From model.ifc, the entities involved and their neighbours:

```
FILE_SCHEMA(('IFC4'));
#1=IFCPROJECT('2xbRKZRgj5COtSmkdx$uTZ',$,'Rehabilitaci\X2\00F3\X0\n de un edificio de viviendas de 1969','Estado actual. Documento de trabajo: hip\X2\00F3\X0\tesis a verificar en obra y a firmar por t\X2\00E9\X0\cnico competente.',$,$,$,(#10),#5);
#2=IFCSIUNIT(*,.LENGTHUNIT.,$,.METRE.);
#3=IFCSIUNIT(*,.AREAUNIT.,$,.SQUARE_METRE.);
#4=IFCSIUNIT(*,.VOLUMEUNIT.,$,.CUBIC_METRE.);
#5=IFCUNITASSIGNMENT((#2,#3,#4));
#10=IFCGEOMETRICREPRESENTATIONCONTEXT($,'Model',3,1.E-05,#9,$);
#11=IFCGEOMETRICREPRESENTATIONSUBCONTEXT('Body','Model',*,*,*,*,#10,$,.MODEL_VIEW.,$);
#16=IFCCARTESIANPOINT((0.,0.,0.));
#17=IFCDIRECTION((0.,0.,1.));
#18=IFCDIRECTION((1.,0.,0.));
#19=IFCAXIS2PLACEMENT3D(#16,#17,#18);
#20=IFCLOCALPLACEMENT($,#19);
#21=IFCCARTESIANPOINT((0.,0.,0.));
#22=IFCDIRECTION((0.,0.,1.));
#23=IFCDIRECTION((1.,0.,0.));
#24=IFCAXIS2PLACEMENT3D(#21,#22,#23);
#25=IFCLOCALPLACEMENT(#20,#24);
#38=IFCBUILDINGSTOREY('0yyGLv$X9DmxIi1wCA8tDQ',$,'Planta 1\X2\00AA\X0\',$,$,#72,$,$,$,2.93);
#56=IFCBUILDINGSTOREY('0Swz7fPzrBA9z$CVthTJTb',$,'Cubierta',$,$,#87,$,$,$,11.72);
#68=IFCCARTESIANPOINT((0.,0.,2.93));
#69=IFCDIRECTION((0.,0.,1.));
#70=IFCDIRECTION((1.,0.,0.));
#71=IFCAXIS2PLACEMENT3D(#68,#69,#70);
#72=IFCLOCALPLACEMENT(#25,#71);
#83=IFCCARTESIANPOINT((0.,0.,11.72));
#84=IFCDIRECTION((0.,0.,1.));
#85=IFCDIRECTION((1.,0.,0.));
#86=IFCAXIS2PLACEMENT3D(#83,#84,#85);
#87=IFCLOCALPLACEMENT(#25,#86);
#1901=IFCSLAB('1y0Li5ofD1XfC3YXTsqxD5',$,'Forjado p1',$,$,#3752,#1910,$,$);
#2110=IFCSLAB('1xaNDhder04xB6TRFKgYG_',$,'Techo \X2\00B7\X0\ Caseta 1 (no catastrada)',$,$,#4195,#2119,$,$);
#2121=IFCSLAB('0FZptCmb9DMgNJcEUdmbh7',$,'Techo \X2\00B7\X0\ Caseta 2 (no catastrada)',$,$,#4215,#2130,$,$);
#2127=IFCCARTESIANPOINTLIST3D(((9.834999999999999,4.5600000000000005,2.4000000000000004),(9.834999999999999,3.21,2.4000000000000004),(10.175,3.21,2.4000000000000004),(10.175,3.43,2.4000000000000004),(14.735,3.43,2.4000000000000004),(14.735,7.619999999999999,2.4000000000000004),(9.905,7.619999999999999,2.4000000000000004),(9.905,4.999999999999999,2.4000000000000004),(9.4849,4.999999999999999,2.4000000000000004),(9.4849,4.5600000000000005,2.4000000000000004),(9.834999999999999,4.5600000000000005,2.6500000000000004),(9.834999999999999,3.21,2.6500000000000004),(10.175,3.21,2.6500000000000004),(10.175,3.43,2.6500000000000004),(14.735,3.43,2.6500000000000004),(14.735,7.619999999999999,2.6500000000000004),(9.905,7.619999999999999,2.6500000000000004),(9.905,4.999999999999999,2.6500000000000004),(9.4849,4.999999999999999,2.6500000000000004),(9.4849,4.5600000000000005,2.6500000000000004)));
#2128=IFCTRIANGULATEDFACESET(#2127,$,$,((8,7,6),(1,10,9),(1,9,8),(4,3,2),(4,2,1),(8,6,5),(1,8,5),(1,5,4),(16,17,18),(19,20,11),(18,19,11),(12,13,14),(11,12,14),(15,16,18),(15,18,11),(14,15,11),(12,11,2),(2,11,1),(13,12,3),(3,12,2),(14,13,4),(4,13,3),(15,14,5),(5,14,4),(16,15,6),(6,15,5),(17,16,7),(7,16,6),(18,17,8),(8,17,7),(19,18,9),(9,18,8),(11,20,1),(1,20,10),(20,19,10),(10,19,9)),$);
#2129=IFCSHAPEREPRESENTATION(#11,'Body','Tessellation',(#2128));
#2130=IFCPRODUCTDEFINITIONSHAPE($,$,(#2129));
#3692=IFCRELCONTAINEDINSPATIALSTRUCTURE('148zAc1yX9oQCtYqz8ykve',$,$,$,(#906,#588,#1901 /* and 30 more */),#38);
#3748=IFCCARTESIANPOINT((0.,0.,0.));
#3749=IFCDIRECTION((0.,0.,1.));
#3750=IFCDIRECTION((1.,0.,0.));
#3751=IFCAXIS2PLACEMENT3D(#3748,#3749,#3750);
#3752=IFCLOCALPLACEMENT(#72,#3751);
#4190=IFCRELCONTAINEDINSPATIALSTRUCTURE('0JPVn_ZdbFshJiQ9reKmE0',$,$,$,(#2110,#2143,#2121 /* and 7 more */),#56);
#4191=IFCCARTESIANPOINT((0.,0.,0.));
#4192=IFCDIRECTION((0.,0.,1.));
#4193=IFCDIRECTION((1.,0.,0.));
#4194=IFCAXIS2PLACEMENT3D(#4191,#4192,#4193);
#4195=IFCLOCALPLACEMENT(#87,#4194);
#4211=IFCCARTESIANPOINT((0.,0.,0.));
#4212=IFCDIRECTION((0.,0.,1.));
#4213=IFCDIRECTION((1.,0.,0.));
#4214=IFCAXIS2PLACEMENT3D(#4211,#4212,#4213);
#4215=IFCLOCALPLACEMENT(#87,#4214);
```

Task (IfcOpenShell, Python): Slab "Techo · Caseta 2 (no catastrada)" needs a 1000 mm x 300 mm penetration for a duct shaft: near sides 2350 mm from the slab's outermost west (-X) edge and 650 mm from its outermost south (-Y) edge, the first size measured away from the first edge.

```python
import numpy as np
import ifcopenshell
import ifcopenshell.api.feature
import ifcopenshell.api.geometry
import ifcopenshell.api.root
import ifcopenshell.geom
import ifcopenshell.util.placement
import ifcopenshell.util.representation
import ifcopenshell.util.shape
import ifcopenshell.util.unit

model = ifcopenshell.open("model.ifc")
unit_scale = ifcopenshell.util.unit.calculate_unit_scale(model)
settings = ifcopenshell.geom.settings()


def volume(element):
    """Net volume in cubic metres, openings subtracted."""
    shape = ifcopenshell.geom.create_shape(settings, element)
    return ifcopenshell.util.shape.get_volume(shape.geometry)


slab = model.by_id(2121)
before = volume(slab)

# Extent in the slab's own axes, in metres. The edges named are its -X and -Y sides.
slab_shape = ifcopenshell.geom.create_shape(settings, slab)
vertices = ifcopenshell.util.shape.get_vertices(slab_shape.geometry)
x_min, y_min, bottom = vertices.min(axis=0)
top = vertices[:, 2].max()

opening = ifcopenshell.api.root.create_entity(model, ifc_class="IfcOpeningElement", name="Duct shaft opening", predefined_type="OPENING")
context = ifcopenshell.util.representation.get_context(model, "Model", "Body", "MODEL_VIEW")
width, depth = 1, 0.3
outline = [(0.0, 0.0), (width, 0.0), (width, depth), (0.0, depth), (0.0, 0.0)]
# Overshoot both faces by 50 mm so the cut is clean.
shape = ifcopenshell.api.geometry.add_slab_representation(
    model, context=context, depth=top - bottom + 0.1, polyline=outline
)
ifcopenshell.api.geometry.assign_representation(model, product=opening, representation=shape)

matrix = ifcopenshell.util.placement.get_local_placement(slab.ObjectPlacement)
matrix[:, 3] = matrix @ np.append(np.array([x_min + 2.35, y_min + 0.65, bottom - 0.05]) / unit_scale, 1.0)
ifcopenshell.api.geometry.edit_object_placement(model, product=opening, matrix=matrix, is_si=False)
ifcopenshell.api.feature.add_feature(model, feature=opening, element=slab)

after = volume(slab)

print(f"slab volume {before:.3f} -> {after:.3f} m3")

model.write("model_updated.ifc")
```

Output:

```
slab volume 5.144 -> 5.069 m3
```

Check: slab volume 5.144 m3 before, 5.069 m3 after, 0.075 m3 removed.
